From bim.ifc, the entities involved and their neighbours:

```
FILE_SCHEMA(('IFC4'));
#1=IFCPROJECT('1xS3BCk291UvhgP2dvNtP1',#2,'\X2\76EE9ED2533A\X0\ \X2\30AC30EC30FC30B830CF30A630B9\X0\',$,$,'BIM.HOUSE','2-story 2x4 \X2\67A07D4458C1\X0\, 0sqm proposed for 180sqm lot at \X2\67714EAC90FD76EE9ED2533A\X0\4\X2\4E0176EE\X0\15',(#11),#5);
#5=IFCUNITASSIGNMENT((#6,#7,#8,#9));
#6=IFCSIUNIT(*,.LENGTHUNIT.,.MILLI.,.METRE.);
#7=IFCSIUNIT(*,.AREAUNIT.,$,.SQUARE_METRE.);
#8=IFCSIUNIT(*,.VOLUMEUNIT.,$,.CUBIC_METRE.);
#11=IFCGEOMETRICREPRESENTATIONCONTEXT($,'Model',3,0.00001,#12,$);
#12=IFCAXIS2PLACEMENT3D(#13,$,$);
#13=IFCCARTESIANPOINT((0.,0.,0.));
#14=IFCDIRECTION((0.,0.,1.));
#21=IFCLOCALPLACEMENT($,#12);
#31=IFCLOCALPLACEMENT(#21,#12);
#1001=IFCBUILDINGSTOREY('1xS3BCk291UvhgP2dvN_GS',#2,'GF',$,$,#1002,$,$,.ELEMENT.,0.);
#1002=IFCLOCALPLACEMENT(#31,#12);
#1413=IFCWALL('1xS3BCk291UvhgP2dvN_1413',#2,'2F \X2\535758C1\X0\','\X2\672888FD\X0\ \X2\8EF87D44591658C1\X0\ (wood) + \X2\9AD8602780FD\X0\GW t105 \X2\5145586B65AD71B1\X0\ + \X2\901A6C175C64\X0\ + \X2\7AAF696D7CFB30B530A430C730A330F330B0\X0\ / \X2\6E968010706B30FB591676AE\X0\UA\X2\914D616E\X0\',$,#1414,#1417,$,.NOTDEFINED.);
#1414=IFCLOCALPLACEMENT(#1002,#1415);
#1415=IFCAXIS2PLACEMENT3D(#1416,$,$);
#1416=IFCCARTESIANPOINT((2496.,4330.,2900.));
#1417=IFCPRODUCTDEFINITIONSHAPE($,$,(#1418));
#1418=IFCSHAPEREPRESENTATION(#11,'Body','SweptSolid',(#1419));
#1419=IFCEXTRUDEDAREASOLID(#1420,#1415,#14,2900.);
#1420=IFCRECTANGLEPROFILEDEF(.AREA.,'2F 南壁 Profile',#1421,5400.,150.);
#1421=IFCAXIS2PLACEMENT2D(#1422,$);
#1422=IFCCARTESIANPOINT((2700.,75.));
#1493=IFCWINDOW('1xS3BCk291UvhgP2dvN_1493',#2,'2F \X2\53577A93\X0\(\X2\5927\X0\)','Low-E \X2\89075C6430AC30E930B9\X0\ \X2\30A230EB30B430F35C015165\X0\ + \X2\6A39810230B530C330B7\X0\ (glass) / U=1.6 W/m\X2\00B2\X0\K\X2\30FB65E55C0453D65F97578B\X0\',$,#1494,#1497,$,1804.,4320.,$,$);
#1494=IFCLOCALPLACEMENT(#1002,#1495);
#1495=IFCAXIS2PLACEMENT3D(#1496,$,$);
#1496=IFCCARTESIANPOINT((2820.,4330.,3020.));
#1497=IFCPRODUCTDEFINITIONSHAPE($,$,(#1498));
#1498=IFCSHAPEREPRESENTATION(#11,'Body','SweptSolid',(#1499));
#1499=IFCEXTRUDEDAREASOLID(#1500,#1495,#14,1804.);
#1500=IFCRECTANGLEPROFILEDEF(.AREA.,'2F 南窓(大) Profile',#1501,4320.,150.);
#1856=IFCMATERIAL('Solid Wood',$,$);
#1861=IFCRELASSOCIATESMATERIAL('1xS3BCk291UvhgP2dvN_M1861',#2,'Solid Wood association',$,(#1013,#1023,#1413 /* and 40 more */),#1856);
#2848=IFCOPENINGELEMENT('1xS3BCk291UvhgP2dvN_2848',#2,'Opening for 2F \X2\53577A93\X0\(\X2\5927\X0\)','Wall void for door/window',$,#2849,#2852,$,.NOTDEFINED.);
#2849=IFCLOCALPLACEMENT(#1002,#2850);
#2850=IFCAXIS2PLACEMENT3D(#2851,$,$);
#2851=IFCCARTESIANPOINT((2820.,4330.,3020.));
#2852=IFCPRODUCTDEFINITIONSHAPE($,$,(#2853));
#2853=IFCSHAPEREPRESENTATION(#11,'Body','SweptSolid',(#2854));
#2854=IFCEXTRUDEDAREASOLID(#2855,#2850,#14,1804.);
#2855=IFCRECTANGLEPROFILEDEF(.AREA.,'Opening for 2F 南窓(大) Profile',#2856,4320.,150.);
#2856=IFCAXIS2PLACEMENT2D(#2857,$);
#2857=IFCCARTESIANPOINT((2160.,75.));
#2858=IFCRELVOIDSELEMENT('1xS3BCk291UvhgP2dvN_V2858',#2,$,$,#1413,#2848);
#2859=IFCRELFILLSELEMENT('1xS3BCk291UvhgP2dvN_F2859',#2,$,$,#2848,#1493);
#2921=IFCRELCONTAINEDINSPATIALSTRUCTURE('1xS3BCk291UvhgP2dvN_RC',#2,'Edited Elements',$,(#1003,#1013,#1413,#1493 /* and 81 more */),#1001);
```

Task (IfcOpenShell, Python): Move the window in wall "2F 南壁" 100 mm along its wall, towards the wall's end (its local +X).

```python
import ifcopenshell
import ifcopenshell.api.geometry
import ifcopenshell.util.placement
import ifcopenshell.util.unit

model = ifcopenshell.open("bim.ifc")
unit_scale = ifcopenshell.util.unit.calculate_unit_scale(model)

window = model.by_guid("1xS3BCk291UvhgP2dvN_1493")
opening = window.FillsVoids[0].RelatingOpeningElement
wall = opening.VoidsElements[0].RelatingBuildingElement

wall_matrix = ifcopenshell.util.placement.get_local_placement(wall.ObjectPlacement)
shift = wall_matrix[:3, 0] * 0.1 / unit_scale
before = ifcopenshell.util.placement.get_local_placement(window.ObjectPlacement)[:3, 3].copy()

# The window is not placed relative to its opening, so move both.
for product in (opening, window):
    matrix = ifcopenshell.util.placement.get_local_placement(product.ObjectPlacement)
    matrix[:3, 3] += shift
    ifcopenshell.api.geometry.edit_object_placement(model, product=product, matrix=matrix, is_si=False)

after = ifcopenshell.util.placement.get_local_placement(window.ObjectPlacement)[:3, 3]
print("window moved by", (after - before).round(3) + 0.0)

model.write("bim-out.ifc")
```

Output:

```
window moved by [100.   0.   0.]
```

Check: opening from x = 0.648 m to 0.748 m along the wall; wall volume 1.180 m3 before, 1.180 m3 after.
